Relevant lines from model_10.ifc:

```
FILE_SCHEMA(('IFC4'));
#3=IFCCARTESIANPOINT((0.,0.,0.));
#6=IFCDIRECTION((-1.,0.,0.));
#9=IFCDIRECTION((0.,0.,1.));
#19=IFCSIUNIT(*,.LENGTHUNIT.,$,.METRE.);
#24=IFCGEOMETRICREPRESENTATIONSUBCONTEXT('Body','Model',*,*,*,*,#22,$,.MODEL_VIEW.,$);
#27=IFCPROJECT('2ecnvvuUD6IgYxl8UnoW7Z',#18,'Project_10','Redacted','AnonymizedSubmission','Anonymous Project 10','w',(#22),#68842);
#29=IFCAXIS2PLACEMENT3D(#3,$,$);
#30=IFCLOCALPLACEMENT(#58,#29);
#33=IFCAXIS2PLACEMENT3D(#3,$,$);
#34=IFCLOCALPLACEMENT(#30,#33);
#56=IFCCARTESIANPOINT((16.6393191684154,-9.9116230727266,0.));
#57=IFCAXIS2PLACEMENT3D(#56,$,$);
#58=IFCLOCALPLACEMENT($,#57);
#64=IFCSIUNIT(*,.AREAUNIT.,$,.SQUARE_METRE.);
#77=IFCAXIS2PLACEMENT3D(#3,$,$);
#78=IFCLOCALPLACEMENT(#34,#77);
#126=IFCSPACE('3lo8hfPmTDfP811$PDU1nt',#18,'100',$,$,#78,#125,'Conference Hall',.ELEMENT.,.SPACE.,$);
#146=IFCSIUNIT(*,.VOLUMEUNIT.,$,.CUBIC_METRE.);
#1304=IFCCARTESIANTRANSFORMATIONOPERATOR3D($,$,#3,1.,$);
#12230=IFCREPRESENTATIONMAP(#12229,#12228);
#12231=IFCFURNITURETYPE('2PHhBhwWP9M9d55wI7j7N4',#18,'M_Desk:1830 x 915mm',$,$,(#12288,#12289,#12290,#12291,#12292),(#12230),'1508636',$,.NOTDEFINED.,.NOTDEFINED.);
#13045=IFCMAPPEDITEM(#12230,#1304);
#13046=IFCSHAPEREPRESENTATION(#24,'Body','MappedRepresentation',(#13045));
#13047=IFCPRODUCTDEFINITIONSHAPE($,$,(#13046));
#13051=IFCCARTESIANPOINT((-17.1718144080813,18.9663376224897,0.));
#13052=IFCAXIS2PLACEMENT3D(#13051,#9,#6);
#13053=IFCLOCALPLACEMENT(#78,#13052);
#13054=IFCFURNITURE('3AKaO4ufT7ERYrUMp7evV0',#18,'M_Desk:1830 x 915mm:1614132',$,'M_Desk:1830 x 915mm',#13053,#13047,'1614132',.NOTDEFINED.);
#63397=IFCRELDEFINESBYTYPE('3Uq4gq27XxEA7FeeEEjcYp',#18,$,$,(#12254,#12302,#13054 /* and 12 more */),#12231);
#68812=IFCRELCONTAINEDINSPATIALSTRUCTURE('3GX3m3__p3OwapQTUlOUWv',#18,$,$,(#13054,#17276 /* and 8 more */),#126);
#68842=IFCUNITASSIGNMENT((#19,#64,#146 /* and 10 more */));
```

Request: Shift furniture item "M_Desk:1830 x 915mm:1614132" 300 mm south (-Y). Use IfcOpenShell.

```python
import ifcopenshell
import ifcopenshell.api.geometry
import ifcopenshell.util.placement
import ifcopenshell.util.unit

model = ifcopenshell.open("model_10.ifc")
unit_scale = ifcopenshell.util.unit.calculate_unit_scale(model)

item = model.by_guid("3AKaO4ufT7ERYrUMp7evV0")
matrix = ifcopenshell.util.placement.get_local_placement(item.ObjectPlacement)
matrix[1, 3] -= 0.3 / unit_scale
ifcopenshell.api.geometry.edit_object_placement(model, product=item, matrix=matrix, is_si=False)

print(ifcopenshell.util.placement.get_local_placement(item.ObjectPlacement).round(3) + 0.0)

model.write("model_10_edited.ifc")
```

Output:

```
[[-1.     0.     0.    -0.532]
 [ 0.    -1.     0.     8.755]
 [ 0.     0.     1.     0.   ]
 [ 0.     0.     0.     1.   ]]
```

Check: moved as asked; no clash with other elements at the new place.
